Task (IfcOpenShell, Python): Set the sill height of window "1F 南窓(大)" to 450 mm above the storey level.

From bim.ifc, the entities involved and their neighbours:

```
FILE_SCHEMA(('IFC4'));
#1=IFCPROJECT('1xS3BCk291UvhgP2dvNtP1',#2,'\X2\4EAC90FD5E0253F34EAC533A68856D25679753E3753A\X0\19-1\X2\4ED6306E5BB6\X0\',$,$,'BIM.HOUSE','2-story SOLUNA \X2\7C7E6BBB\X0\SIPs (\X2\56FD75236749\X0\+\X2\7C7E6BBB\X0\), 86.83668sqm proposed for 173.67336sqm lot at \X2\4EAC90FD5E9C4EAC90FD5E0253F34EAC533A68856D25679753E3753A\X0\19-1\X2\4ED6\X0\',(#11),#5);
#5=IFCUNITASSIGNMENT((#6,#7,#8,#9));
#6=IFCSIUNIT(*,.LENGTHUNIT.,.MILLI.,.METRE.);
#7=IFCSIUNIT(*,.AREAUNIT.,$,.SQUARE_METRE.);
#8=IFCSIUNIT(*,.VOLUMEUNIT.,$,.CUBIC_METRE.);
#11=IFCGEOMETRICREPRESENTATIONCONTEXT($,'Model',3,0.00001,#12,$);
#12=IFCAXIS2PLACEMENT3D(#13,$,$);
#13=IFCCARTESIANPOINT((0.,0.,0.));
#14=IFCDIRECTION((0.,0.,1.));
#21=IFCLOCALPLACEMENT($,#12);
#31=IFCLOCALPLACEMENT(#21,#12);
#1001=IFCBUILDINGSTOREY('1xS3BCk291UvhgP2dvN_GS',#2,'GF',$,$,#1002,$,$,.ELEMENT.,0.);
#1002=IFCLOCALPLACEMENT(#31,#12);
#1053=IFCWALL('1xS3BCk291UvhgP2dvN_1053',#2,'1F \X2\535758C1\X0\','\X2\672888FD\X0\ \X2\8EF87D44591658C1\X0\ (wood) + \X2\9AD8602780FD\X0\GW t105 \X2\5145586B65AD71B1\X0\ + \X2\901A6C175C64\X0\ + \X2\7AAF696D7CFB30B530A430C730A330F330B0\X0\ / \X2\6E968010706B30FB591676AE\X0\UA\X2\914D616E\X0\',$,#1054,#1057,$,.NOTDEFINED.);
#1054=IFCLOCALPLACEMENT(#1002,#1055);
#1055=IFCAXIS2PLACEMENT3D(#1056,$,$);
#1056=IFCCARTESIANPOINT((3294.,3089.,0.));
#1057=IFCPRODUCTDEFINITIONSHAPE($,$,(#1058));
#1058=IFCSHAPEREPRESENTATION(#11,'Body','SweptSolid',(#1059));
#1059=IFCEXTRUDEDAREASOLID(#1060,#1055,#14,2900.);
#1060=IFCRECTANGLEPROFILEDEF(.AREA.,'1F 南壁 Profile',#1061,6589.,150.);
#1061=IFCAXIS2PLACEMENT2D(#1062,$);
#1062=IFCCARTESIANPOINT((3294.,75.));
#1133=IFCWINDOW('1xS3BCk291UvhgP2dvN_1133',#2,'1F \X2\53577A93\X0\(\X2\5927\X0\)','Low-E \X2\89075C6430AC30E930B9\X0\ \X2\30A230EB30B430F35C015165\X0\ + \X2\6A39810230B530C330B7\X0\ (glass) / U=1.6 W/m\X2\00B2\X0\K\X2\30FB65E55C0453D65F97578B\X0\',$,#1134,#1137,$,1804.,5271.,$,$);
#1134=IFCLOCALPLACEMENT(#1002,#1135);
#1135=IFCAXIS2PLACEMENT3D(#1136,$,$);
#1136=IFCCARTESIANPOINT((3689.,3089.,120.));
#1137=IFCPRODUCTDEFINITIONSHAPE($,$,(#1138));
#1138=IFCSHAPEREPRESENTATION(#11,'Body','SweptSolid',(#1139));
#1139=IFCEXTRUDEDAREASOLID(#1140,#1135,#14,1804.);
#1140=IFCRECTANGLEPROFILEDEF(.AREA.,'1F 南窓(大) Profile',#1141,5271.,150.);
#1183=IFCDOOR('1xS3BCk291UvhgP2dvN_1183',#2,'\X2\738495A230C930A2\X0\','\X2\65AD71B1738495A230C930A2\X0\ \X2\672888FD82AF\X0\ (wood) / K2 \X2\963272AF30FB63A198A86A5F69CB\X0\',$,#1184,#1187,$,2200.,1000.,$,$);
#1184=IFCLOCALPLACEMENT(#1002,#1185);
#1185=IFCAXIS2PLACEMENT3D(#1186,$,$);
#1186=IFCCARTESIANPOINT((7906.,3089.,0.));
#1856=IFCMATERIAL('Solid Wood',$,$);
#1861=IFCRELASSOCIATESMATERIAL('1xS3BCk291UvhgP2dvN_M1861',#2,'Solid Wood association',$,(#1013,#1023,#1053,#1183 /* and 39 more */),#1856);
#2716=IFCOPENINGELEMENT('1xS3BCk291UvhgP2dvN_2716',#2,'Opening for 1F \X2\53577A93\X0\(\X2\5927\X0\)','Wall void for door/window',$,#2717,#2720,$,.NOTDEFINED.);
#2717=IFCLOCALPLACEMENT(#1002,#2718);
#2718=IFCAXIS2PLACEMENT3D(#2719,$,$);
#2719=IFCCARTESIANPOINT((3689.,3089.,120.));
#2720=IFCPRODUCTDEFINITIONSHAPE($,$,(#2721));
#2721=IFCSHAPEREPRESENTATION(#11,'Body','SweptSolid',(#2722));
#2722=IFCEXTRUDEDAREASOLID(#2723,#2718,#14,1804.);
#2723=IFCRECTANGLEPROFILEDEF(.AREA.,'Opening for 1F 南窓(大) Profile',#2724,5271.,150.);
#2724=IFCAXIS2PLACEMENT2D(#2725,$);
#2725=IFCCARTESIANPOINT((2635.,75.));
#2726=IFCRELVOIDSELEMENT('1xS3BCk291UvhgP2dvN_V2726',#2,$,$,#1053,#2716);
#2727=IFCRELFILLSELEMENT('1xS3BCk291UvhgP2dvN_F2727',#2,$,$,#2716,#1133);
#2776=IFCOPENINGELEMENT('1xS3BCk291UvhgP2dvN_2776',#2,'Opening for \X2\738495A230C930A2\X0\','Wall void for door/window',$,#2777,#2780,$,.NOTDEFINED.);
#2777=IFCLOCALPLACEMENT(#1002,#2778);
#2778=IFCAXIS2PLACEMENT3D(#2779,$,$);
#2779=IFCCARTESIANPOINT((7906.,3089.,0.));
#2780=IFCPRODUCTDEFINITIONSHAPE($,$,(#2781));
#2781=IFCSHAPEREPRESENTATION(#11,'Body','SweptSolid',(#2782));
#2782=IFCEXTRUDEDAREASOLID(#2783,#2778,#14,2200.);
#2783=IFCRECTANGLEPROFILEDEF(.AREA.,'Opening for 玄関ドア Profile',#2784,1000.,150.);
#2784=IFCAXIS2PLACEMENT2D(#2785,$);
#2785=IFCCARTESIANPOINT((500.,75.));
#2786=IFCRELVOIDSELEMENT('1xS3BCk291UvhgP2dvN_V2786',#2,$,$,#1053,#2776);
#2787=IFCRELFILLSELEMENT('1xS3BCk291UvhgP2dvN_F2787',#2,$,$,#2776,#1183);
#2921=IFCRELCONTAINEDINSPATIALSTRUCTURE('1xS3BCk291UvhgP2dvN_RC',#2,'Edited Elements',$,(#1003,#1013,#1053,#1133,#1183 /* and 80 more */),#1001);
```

```python
import numpy as np
import ifcopenshell
import ifcopenshell.api.geometry
import ifcopenshell.geom
import ifcopenshell.util.element
import ifcopenshell.util.placement
import ifcopenshell.util.shape
import ifcopenshell.util.unit

model = ifcopenshell.open("bim.ifc")
unit_scale = ifcopenshell.util.unit.calculate_unit_scale(model)

window = model.by_id(1133)
opening = window.FillsVoids[0].RelatingOpeningElement
storey = ifcopenshell.util.element.get_container(window, ifc_class="IfcBuildingStorey")
level = ifcopenshell.util.placement.get_local_placement(storey.ObjectPlacement)[2, 3]

# The opening's origin need not be at the sill, so measure its lowest point.
shape = ifcopenshell.geom.create_shape(ifcopenshell.geom.settings(), opening)
bottom = ifcopenshell.util.shape.get_shape_bottom_elevation(shape, shape.geometry) / unit_scale
dz = level + 450.0 - bottom

shift = np.array([0.0, 0.0, dz])
# The window is not placed relative to its opening, so move both.
for product in (opening, window):
    matrix = ifcopenshell.util.placement.get_local_placement(product.ObjectPlacement)
    matrix[:3, 3] += shift
    ifcopenshell.api.geometry.edit_object_placement(model, product=product, matrix=matrix, is_si=False)

print(f"moved by {dz * unit_scale:+.3f} m")

model.write("bim_v2.ifc")
```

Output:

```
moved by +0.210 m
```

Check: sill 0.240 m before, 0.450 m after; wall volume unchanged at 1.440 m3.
